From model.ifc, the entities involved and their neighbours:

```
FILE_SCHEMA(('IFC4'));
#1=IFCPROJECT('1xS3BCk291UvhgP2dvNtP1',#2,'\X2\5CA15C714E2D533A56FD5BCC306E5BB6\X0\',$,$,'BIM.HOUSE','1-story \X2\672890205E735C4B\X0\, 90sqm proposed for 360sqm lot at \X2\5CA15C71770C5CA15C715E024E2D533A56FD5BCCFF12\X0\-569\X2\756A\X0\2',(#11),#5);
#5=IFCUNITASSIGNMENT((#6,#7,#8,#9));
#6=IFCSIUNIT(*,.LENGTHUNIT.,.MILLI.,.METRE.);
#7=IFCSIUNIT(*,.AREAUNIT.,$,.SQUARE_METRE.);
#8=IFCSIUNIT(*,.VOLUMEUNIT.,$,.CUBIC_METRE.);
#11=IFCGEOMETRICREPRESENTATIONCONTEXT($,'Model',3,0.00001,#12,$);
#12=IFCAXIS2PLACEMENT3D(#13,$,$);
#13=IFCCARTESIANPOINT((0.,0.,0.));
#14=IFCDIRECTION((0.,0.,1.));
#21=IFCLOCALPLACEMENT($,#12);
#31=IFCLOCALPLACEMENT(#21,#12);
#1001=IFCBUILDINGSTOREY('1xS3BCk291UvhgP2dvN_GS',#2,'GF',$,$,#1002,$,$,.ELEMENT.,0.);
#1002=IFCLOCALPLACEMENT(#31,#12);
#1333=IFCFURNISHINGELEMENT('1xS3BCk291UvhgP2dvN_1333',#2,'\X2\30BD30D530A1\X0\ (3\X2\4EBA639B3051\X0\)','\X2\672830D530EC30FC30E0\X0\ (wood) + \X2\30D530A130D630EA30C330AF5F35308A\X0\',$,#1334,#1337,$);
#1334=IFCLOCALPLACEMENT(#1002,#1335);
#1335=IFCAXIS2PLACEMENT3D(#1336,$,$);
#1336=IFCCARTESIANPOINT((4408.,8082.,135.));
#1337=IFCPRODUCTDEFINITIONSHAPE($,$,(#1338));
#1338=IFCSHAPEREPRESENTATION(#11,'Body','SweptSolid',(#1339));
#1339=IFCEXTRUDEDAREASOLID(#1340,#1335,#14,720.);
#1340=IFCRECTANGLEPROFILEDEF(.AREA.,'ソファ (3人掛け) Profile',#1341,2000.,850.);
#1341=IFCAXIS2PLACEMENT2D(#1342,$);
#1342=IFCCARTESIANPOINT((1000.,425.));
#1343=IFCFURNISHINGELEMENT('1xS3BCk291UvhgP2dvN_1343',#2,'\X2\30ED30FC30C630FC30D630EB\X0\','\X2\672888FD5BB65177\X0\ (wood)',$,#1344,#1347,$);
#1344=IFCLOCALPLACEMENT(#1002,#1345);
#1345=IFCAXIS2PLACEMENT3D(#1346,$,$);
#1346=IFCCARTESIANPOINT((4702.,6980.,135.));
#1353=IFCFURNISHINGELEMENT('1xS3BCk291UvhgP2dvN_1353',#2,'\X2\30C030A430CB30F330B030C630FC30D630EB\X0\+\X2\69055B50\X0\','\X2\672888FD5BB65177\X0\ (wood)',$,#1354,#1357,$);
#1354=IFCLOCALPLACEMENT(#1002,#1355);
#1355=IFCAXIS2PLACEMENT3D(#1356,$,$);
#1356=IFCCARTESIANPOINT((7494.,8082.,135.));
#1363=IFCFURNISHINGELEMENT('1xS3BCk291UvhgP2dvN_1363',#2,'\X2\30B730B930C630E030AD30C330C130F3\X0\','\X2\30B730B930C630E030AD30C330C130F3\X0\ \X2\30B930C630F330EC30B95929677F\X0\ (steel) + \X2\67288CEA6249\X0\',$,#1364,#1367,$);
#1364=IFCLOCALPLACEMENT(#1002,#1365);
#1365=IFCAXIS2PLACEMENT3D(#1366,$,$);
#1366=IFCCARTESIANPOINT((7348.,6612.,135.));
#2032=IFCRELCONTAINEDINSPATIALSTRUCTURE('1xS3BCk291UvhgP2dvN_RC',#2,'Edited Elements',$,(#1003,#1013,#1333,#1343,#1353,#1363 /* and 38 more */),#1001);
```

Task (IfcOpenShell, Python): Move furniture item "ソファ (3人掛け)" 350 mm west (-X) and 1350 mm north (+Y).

```python
import ifcopenshell
import ifcopenshell.api.geometry
import ifcopenshell.util.placement
import ifcopenshell.util.unit

model = ifcopenshell.open("model.ifc")
unit_scale = ifcopenshell.util.unit.calculate_unit_scale(model)

item = model.by_guid("1xS3BCk291UvhgP2dvN_1333")
matrix = ifcopenshell.util.placement.get_local_placement(item.ObjectPlacement)
matrix[0, 3] -= 0.35 / unit_scale
matrix[1, 3] += 1.35 / unit_scale
ifcopenshell.api.geometry.edit_object_placement(model, product=item, matrix=matrix, is_si=False)

print(ifcopenshell.util.placement.get_local_placement(item.ObjectPlacement).round(3) + 0.0)

model.write("model-out.ifc")
```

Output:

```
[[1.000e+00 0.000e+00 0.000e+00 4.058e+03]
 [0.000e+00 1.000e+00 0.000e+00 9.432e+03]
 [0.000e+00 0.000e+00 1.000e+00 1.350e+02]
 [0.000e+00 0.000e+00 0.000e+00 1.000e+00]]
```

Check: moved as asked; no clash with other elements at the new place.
